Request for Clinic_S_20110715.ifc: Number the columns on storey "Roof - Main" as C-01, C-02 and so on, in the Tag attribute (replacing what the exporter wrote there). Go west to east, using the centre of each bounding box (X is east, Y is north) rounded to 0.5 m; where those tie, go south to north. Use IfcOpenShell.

First a look at what the model holds.

```python
import ifcopenshell
import ifcopenshell.util.element
import ifcopenshell.util.placement

model = ifcopenshell.open("Clinic_S_20110715.ifc")
print(model.schema)
storey = next(s for s in model.by_type("IfcBuildingStorey") if s.Name == "Roof - Main")
columns = [e for e in ifcopenshell.util.element.get_decomposition(storey) if e.is_a("IfcColumn")]
for e in sorted(columns, key=lambda e: e.id()):
    origin = ifcopenshell.util.placement.get_local_placement(e.ObjectPlacement)[:3, 3]
    print(e.id(), e.Tag, e.Name, origin.round(2) + 0.0, sep=" | ")
```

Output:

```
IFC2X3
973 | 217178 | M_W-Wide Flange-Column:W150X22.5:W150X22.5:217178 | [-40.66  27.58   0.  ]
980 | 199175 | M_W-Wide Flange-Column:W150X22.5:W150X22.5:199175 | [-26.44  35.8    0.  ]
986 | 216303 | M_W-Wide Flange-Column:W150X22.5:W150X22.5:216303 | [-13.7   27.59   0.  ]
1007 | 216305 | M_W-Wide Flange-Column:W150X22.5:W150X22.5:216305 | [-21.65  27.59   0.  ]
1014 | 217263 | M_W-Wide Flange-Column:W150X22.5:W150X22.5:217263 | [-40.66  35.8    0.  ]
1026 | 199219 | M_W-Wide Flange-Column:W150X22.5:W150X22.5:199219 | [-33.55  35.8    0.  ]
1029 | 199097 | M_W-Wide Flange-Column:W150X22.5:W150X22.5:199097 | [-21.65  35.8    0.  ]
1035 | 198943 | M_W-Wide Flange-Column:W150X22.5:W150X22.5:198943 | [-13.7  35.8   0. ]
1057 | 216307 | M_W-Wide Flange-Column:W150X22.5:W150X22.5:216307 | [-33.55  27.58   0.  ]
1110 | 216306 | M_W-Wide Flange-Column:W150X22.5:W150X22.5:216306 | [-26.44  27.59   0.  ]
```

```python
import ifcopenshell
import ifcopenshell.geom
import ifcopenshell.util.element
import ifcopenshell.util.shape

model = ifcopenshell.open("Clinic_S_20110715.ifc")
settings = ifcopenshell.geom.settings()
settings.set("use-world-coords", True)


def centre(element):
    shape = ifcopenshell.geom.create_shape(settings, element)
    return ifcopenshell.util.shape.get_bbox_centroid(shape.geometry)


storey = next(s for s in model.by_type("IfcBuildingStorey") if s.Name == "Roof - Main")
columns = [e for e in ifcopenshell.util.element.get_decomposition(storey) if e.is_a("IfcColumn")]

# Insertion points can sit at a corner or the storey origin, so sort by the geometry (in metres).
centres = {e: centre(e) for e in columns}
columns.sort(key=lambda e: (round(centres[e][0] / 0.5), centres[e][1]))

for i, e in enumerate(columns, start=1):
    number = f"C-{i:02d}"
    e.Tag = number
    print(e.id(), number)

model.write("Clinic_S_20110715_v2.ifc")
```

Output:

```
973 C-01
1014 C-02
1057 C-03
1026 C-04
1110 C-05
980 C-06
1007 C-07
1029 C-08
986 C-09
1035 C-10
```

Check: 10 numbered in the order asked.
